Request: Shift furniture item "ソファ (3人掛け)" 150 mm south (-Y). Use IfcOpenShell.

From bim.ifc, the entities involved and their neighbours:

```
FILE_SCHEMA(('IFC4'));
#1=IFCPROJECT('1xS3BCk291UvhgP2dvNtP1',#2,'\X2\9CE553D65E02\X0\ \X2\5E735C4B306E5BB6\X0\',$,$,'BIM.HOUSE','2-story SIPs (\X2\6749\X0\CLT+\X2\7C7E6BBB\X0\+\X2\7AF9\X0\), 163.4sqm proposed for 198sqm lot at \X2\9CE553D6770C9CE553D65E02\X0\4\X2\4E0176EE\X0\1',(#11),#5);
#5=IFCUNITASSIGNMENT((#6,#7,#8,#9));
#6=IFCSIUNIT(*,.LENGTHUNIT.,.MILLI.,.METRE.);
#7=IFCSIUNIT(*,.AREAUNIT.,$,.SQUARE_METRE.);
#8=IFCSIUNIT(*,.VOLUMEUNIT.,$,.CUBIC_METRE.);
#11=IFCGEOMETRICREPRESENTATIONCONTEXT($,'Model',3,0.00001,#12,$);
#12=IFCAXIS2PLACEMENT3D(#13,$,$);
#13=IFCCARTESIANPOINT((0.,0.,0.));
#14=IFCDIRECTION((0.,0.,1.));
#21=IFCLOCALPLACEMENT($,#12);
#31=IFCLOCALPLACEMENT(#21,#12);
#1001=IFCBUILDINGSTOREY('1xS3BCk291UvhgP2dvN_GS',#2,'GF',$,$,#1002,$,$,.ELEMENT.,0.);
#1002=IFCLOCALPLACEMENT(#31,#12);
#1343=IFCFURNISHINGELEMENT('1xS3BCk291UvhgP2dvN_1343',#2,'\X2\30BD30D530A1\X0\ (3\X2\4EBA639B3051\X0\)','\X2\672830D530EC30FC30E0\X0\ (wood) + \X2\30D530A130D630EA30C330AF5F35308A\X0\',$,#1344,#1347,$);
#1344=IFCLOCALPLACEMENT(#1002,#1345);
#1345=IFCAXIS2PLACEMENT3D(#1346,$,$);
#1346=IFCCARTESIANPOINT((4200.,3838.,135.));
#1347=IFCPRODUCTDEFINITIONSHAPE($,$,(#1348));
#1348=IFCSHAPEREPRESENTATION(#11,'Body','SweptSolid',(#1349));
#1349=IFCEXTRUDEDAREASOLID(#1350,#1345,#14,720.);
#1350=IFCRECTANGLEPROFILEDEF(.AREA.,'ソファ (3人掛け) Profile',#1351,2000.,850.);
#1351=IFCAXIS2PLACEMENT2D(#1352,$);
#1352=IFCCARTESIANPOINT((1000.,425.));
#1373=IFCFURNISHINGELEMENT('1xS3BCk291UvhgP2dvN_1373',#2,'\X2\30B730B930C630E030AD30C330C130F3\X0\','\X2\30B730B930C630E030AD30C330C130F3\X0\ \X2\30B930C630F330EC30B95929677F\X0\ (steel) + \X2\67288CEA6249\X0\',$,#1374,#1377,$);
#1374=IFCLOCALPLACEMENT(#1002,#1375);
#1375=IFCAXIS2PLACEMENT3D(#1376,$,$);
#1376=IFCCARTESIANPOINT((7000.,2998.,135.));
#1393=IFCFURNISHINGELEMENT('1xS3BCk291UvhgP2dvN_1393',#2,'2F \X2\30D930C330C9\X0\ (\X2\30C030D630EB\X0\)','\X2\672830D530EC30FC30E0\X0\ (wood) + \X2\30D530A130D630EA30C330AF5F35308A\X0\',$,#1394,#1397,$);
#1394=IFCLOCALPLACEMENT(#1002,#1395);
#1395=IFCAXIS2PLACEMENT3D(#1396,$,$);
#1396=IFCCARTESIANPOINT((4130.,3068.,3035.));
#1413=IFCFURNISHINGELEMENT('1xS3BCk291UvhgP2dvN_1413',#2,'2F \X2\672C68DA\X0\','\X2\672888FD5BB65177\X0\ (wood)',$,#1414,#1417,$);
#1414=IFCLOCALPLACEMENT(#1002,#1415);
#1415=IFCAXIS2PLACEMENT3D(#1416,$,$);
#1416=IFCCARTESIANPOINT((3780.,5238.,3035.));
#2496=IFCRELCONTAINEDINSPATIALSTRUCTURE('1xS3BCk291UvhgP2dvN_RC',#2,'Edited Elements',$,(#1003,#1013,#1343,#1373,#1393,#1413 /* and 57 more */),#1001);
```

```python
import ifcopenshell
import ifcopenshell.api.geometry
import ifcopenshell.util.placement

model = ifcopenshell.open("bim.ifc")

item = model.by_guid("1xS3BCk291UvhgP2dvN_1343")
matrix = ifcopenshell.util.placement.get_local_placement(item.ObjectPlacement)
matrix[1, 3] -= 150.0
ifcopenshell.api.geometry.edit_object_placement(model, product=item, matrix=matrix, is_si=False)

print(ifcopenshell.util.placement.get_local_placement(item.ObjectPlacement).round(3) + 0.0)

model.write("bim-out.ifc")
```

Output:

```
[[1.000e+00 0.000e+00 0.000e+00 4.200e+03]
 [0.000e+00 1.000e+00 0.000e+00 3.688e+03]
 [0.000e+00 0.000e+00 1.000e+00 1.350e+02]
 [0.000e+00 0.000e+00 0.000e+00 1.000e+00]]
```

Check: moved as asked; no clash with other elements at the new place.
